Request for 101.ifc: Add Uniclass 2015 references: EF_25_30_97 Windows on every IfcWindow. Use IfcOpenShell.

First a look at what the model holds.

```python
import ifcopenshell

model = ifcopenshell.open("101.ifc")
print(model.schema)
print("classifications:", [c.Name for c in model.by_type("IfcClassification")])
for ifc_class in ("IfcDoor", "IfcRoof", "IfcStair", "IfcWall", "IfcWindow"):
    print(ifc_class, len(model.by_type(ifc_class)))
```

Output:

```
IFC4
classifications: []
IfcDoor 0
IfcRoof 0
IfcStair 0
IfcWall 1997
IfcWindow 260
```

```python
import ifcopenshell
import ifcopenshell.api.classification

model = ifcopenshell.open("101.ifc")

system = ifcopenshell.api.classification.add_classification(model, classification="Uniclass 2015")

codes = {
    "IfcWindow": ("EF_25_30_97", "Windows"),
}
for ifc_class, (code, name) in codes.items():
    products = model.by_type(ifc_class)
    ifcopenshell.api.classification.add_reference(
        model, products=products, classification=system, identification=code, name=name
    )
    print(code, len(products))

model.write("101_v2.ifc")
```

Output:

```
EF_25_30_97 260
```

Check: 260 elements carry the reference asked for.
